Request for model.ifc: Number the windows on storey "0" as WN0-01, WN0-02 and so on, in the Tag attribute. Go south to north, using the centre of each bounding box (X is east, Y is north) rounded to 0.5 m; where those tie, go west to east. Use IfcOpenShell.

First a look at what the model holds.

```python
import ifcopenshell
import ifcopenshell.util.element
import ifcopenshell.util.placement

model = ifcopenshell.open("model.ifc")
print(model.schema)
storey = next(s for s in model.by_type("IfcBuildingStorey") if s.Name == "0")
windows = [e for e in ifcopenshell.util.element.get_decomposition(storey) if e.is_a("IfcWindow")]
for e in sorted(windows, key=lambda e: e.id()):
    origin = ifcopenshell.util.placement.get_local_placement(e.ObjectPlacement)[:3, 3]
    print(e.id(), e.Tag, e.Name, origin.round(2) + 0.0, sep=" | ")
```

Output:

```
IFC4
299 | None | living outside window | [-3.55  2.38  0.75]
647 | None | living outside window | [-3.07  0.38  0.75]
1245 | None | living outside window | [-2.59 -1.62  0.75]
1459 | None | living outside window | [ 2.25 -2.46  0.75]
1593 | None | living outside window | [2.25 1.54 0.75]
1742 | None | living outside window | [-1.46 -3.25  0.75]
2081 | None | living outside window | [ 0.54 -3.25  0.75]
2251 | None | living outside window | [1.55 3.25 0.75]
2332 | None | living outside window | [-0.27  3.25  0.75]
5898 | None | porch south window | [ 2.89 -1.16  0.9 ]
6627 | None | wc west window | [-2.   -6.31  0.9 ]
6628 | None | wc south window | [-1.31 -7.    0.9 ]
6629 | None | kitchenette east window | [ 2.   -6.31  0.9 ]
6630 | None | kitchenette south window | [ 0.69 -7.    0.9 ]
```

```python
import ifcopenshell
import ifcopenshell.geom
import ifcopenshell.util.element
import ifcopenshell.util.shape

model = ifcopenshell.open("model.ifc")
settings = ifcopenshell.geom.settings()
settings.set("use-world-coords", True)


def centre(element):
    shape = ifcopenshell.geom.create_shape(settings, element)
    return ifcopenshell.util.shape.get_bbox_centroid(shape.geometry)


storey = next(s for s in model.by_type("IfcBuildingStorey") if s.Name == "0")
windows = [e for e in ifcopenshell.util.element.get_decomposition(storey) if e.is_a("IfcWindow")]

# Insertion points can sit at a corner or the storey origin, so sort by the geometry (in metres).
centres = {e: centre(e) for e in windows}
windows.sort(key=lambda e: (round(centres[e][1] / 0.5), centres[e][0]))

for i, e in enumerate(windows, start=1):
    number = f"WN0-{i:02d}"
    e.Tag = number
    print(e.id(), number)

model.write("model_v2.ifc")
```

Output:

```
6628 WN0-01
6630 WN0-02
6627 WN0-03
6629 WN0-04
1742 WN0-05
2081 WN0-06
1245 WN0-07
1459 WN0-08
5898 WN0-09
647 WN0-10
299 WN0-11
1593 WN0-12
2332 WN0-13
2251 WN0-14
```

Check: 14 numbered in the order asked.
